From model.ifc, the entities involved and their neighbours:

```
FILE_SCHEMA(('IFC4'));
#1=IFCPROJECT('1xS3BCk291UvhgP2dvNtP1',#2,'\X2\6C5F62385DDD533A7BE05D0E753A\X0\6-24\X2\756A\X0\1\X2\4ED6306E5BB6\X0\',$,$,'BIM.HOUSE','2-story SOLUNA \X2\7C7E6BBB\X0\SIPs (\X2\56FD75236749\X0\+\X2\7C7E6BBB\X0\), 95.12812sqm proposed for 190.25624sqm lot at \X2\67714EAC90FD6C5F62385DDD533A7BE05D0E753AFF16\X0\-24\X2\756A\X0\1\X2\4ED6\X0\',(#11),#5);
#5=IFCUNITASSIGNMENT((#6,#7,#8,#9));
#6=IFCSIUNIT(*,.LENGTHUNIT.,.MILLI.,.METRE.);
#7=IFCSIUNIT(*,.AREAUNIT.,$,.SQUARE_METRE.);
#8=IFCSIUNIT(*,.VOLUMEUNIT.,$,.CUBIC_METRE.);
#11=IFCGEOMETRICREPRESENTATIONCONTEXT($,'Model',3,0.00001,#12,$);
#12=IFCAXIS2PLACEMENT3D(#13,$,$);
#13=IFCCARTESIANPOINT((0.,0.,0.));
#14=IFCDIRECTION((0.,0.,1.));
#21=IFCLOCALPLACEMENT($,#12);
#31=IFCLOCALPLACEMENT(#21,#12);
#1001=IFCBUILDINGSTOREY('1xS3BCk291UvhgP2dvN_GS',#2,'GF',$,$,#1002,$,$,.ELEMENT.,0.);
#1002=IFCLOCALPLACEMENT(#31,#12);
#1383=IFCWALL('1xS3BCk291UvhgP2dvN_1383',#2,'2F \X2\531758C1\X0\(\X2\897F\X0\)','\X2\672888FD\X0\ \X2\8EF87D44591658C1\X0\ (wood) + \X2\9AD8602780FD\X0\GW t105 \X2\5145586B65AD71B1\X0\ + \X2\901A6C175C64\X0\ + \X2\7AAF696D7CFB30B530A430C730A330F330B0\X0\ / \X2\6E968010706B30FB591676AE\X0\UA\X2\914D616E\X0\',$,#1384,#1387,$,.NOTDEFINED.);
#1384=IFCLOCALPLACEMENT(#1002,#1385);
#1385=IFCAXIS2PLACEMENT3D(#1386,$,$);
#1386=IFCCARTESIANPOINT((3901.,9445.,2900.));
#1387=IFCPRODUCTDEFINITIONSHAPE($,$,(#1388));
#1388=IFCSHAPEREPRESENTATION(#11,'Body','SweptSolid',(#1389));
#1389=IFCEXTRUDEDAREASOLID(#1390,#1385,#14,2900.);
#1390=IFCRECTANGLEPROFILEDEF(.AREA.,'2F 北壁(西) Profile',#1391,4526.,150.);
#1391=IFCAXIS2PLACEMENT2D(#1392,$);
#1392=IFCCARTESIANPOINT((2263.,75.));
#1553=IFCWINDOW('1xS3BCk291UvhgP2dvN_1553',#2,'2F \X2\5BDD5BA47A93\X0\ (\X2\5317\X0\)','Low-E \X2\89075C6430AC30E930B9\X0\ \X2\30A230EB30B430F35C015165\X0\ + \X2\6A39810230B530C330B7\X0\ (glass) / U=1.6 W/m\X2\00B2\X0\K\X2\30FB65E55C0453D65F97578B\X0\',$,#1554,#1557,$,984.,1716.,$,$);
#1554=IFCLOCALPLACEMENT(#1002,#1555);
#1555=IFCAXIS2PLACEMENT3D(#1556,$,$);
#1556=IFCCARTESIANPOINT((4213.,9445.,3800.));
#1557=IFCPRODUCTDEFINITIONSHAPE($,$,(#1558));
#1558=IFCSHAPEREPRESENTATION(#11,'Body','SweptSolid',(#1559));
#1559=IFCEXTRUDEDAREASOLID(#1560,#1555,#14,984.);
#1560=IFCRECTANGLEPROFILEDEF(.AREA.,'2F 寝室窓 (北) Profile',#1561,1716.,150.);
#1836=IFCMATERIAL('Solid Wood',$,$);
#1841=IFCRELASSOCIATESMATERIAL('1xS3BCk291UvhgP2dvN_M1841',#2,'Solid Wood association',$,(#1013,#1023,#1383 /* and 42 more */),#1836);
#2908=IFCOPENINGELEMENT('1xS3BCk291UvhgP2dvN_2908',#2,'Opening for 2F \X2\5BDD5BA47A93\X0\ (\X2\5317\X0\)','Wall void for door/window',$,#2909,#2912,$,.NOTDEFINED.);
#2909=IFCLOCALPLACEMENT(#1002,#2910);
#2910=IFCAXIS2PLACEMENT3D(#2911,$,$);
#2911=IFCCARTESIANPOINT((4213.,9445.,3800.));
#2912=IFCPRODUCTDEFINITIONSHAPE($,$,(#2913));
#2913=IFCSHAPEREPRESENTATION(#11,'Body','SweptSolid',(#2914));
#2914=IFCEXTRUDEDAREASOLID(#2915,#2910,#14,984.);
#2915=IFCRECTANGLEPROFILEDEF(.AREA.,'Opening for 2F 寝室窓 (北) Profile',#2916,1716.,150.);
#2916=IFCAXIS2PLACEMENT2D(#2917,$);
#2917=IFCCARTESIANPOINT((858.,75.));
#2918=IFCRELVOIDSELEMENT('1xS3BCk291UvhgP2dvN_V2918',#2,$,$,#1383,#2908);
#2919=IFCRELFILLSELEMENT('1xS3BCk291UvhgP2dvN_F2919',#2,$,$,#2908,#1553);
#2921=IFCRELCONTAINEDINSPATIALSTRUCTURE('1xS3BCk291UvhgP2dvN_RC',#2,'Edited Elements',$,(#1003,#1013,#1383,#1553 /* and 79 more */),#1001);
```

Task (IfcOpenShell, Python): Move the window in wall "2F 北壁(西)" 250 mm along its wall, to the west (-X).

```python
import ifcopenshell
import ifcopenshell.api.geometry
import ifcopenshell.util.placement
import ifcopenshell.util.unit

model = ifcopenshell.open("model.ifc")
unit_scale = ifcopenshell.util.unit.calculate_unit_scale(model)

window = model.by_guid("1xS3BCk291UvhgP2dvN_1553")
opening = window.FillsVoids[0].RelatingOpeningElement
wall = opening.VoidsElements[0].RelatingBuildingElement

wall_matrix = ifcopenshell.util.placement.get_local_placement(wall.ObjectPlacement)
shift = wall_matrix[:3, 0] * -0.25 / unit_scale
before = ifcopenshell.util.placement.get_local_placement(window.ObjectPlacement)[:3, 3].copy()

# The window is not placed relative to its opening, so move both.
for product in (opening, window):
    matrix = ifcopenshell.util.placement.get_local_placement(product.ObjectPlacement)
    matrix[:3, 3] += shift
    ifcopenshell.api.geometry.edit_object_placement(model, product=product, matrix=matrix, is_si=False)

after = ifcopenshell.util.placement.get_local_placement(window.ObjectPlacement)[:3, 3]
print("window moved by", (after - before).round(3) + 0.0)

model.write("model-out.ifc")
```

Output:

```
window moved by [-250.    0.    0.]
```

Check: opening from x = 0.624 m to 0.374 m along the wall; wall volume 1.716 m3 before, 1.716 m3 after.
